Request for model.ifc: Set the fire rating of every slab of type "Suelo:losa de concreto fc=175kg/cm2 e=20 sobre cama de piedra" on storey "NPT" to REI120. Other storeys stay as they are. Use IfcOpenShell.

First a look at what the model holds.

```python
import ifcopenshell
import ifcopenshell.util.element

model = ifcopenshell.open("model.ifc")
print(model.schema)
storey = next(s for s in model.by_type("IfcBuildingStorey") if s.Name == "NPT")
slabs = [e for e in ifcopenshell.util.element.get_decomposition(storey) if e.is_a("IfcSlab")]
seen = {}
for e in slabs:
    element_type = ifcopenshell.util.element.get_type(e)
    key = (element_type.Name if element_type != e and element_type else None, ifcopenshell.util.element.get_pset(e, "Pset_SlabCommon", "FireRating"))
    seen[key] = seen.get(key, 0) + 1
for (name, value), count in sorted(seen.items(), key=str):
    print(count, "x", name, "|", value)
```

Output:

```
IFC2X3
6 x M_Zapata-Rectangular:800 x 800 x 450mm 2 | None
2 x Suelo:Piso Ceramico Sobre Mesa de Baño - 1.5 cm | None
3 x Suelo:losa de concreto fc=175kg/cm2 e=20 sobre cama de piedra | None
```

```python
import ifcopenshell
import ifcopenshell.api.pset
import ifcopenshell.util.element

model = ifcopenshell.open("model.ifc")

storey = next(s for s in model.by_type("IfcBuildingStorey") if s.Name == "NPT")
slabs = [e for e in ifcopenshell.util.element.get_decomposition(storey) if e.is_a("IfcSlab")]

count = 0
for e in slabs:
    element_type = ifcopenshell.util.element.get_type(e)
    if element_type in (None, e) or element_type.Name != "Suelo:losa de concreto fc=175kg/cm2 e=20 sobre cama de piedra":
        continue
    # add_pset returns the element's existing set when there is one.
    pset = ifcopenshell.api.pset.add_pset(model, product=e, name="Pset_SlabCommon")
    ifcopenshell.api.pset.edit_pset(model, pset=pset, properties={"FireRating": "REI120"})
    count += 1

print(count, "slabs updated")

model.write("model_rev.ifc")
```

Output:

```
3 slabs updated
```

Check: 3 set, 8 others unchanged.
